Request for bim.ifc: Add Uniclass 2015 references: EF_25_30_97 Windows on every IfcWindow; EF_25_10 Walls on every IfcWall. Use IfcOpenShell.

First a look at what the model holds.

```python
import ifcopenshell

model = ifcopenshell.open("bim.ifc")
print(model.schema)
print("classifications:", [c.Name for c in model.by_type("IfcClassification")])
for ifc_class in ("IfcDoor", "IfcRoof", "IfcStair", "IfcWall", "IfcWindow"):
    print(ifc_class, len(model.by_type(ifc_class)))
```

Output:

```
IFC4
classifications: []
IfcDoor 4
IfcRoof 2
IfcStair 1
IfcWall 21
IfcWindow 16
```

```python
import ifcopenshell
import ifcopenshell.api.classification

model = ifcopenshell.open("bim.ifc")

system = ifcopenshell.api.classification.add_classification(model, classification="Uniclass 2015")

codes = {
    "IfcWindow": ("EF_25_30_97", "Windows"),
    "IfcWall": ("EF_25_10", "Walls"),
}
for ifc_class, (code, name) in codes.items():
    products = model.by_type(ifc_class)
    ifcopenshell.api.classification.add_reference(
        model, products=products, classification=system, identification=code, name=name
    )
    print(code, len(products))

model.write("bim_rev.ifc")
```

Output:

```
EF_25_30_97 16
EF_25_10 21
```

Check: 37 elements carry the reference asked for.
